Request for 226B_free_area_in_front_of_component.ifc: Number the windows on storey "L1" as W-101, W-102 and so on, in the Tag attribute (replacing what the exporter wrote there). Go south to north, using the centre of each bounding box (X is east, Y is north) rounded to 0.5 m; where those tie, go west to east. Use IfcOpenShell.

First a look at what the model holds.

```python
import ifcopenshell
import ifcopenshell.util.element
import ifcopenshell.util.placement

model = ifcopenshell.open("226B_free_area_in_front_of_component.ifc")
print(model.schema)
storey = next(s for s in model.by_type("IfcBuildingStorey") if s.Name == "L1")
windows = [e for e in ifcopenshell.util.element.get_decomposition(storey) if e.is_a("IfcWindow")]
for e in sorted(windows, key=lambda e: e.id()):
    origin = ifcopenshell.util.placement.get_local_placement(e.ObjectPlacement)[:3, 3]
    print(e.id(), e.Tag, e.Name, origin.round(2) + 0.0, sep=" | ")
```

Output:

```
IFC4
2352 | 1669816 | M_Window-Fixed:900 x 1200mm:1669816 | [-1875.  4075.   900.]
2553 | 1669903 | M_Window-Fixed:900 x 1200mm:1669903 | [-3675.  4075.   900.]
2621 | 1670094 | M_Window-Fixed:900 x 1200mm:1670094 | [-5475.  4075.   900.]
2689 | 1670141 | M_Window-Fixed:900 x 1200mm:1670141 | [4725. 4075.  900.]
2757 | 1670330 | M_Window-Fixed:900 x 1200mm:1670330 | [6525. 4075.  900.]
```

```python
import ifcopenshell
import ifcopenshell.geom
import ifcopenshell.util.element
import ifcopenshell.util.shape

model = ifcopenshell.open("226B_free_area_in_front_of_component.ifc")
settings = ifcopenshell.geom.settings()
settings.set("use-world-coords", True)


def centre(element):
    shape = ifcopenshell.geom.create_shape(settings, element)
    return ifcopenshell.util.shape.get_bbox_centroid(shape.geometry)


storey = next(s for s in model.by_type("IfcBuildingStorey") if s.Name == "L1")
windows = [e for e in ifcopenshell.util.element.get_decomposition(storey) if e.is_a("IfcWindow")]

# Insertion points can sit at a corner or the storey origin, so sort by the geometry (in metres).
centres = {e: centre(e) for e in windows}
windows.sort(key=lambda e: (round(centres[e][1] / 0.5), centres[e][0]))

for i, e in enumerate(windows, start=1):
    number = f"W-1{i:02d}"
    e.Tag = number
    print(e.id(), number)

model.write("226B_free_area_in_front_of_component_v2.ifc")
```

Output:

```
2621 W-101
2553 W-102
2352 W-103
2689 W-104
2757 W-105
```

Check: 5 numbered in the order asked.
